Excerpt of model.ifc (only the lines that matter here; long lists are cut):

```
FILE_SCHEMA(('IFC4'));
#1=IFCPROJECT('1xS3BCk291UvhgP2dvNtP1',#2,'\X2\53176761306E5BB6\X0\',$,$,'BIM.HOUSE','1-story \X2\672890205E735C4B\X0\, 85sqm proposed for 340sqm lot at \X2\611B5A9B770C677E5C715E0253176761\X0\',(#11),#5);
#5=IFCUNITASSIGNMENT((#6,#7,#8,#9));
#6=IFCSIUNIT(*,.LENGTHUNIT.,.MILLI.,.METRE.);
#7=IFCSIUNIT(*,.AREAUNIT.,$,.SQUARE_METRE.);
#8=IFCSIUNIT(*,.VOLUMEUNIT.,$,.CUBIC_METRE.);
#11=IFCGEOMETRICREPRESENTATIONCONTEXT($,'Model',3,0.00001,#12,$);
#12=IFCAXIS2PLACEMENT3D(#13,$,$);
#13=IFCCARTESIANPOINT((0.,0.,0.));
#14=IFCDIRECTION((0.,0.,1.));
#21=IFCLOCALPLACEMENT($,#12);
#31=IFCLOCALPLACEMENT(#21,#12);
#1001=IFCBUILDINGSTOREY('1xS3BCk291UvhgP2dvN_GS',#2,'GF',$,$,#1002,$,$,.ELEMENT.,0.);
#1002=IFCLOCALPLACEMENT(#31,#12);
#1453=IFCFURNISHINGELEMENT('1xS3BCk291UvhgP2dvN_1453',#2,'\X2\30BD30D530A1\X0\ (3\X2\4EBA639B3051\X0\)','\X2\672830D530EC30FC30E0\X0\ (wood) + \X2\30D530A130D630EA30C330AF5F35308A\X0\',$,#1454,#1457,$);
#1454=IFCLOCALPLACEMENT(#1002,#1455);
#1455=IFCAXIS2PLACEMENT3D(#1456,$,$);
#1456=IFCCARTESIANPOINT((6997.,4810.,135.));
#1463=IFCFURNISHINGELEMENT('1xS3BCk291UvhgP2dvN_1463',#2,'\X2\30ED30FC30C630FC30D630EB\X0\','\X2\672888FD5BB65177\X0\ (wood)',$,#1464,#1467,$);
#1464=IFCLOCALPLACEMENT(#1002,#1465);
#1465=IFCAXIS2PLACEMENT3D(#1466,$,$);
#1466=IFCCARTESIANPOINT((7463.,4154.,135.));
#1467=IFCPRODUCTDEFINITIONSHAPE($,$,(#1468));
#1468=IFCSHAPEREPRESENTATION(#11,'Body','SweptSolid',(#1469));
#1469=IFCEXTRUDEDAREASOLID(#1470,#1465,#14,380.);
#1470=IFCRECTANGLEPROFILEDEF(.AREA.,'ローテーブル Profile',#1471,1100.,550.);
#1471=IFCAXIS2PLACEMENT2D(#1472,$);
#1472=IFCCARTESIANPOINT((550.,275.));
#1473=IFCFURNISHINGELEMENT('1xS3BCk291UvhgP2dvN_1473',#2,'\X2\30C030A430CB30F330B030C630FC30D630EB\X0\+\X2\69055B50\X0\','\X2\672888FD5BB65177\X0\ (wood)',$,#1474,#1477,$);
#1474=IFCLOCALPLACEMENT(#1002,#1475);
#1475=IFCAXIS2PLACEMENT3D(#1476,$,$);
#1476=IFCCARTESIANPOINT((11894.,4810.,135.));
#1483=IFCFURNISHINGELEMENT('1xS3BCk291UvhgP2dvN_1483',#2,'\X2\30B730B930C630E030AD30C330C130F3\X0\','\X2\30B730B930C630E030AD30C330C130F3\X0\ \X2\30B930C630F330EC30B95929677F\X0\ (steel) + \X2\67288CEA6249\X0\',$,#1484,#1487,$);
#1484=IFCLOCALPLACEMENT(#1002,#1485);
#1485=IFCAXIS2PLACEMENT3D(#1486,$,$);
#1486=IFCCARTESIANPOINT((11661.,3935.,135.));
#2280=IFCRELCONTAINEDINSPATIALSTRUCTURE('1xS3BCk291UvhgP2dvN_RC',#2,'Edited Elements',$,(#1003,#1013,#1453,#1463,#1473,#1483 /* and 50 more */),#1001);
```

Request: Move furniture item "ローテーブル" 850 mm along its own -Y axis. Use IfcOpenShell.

```python
import ifcopenshell
import ifcopenshell.api.geometry
import ifcopenshell.util.placement
import ifcopenshell.util.unit

model = ifcopenshell.open("model.ifc")
unit_scale = ifcopenshell.util.unit.calculate_unit_scale(model)

item = model.by_guid("1xS3BCk291UvhgP2dvN_1463")
matrix = ifcopenshell.util.placement.get_local_placement(item.ObjectPlacement)
matrix[:3, 3] -= matrix[:3, 1] * 0.85 / unit_scale
ifcopenshell.api.geometry.edit_object_placement(model, product=item, matrix=matrix, is_si=False)

print(ifcopenshell.util.placement.get_local_placement(item.ObjectPlacement).round(3) + 0.0)

model.write("model_rev.ifc")
```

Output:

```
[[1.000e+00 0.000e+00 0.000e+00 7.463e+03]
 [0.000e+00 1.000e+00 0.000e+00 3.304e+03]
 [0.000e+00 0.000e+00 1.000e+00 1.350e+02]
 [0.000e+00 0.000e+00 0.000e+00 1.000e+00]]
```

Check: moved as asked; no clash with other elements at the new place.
